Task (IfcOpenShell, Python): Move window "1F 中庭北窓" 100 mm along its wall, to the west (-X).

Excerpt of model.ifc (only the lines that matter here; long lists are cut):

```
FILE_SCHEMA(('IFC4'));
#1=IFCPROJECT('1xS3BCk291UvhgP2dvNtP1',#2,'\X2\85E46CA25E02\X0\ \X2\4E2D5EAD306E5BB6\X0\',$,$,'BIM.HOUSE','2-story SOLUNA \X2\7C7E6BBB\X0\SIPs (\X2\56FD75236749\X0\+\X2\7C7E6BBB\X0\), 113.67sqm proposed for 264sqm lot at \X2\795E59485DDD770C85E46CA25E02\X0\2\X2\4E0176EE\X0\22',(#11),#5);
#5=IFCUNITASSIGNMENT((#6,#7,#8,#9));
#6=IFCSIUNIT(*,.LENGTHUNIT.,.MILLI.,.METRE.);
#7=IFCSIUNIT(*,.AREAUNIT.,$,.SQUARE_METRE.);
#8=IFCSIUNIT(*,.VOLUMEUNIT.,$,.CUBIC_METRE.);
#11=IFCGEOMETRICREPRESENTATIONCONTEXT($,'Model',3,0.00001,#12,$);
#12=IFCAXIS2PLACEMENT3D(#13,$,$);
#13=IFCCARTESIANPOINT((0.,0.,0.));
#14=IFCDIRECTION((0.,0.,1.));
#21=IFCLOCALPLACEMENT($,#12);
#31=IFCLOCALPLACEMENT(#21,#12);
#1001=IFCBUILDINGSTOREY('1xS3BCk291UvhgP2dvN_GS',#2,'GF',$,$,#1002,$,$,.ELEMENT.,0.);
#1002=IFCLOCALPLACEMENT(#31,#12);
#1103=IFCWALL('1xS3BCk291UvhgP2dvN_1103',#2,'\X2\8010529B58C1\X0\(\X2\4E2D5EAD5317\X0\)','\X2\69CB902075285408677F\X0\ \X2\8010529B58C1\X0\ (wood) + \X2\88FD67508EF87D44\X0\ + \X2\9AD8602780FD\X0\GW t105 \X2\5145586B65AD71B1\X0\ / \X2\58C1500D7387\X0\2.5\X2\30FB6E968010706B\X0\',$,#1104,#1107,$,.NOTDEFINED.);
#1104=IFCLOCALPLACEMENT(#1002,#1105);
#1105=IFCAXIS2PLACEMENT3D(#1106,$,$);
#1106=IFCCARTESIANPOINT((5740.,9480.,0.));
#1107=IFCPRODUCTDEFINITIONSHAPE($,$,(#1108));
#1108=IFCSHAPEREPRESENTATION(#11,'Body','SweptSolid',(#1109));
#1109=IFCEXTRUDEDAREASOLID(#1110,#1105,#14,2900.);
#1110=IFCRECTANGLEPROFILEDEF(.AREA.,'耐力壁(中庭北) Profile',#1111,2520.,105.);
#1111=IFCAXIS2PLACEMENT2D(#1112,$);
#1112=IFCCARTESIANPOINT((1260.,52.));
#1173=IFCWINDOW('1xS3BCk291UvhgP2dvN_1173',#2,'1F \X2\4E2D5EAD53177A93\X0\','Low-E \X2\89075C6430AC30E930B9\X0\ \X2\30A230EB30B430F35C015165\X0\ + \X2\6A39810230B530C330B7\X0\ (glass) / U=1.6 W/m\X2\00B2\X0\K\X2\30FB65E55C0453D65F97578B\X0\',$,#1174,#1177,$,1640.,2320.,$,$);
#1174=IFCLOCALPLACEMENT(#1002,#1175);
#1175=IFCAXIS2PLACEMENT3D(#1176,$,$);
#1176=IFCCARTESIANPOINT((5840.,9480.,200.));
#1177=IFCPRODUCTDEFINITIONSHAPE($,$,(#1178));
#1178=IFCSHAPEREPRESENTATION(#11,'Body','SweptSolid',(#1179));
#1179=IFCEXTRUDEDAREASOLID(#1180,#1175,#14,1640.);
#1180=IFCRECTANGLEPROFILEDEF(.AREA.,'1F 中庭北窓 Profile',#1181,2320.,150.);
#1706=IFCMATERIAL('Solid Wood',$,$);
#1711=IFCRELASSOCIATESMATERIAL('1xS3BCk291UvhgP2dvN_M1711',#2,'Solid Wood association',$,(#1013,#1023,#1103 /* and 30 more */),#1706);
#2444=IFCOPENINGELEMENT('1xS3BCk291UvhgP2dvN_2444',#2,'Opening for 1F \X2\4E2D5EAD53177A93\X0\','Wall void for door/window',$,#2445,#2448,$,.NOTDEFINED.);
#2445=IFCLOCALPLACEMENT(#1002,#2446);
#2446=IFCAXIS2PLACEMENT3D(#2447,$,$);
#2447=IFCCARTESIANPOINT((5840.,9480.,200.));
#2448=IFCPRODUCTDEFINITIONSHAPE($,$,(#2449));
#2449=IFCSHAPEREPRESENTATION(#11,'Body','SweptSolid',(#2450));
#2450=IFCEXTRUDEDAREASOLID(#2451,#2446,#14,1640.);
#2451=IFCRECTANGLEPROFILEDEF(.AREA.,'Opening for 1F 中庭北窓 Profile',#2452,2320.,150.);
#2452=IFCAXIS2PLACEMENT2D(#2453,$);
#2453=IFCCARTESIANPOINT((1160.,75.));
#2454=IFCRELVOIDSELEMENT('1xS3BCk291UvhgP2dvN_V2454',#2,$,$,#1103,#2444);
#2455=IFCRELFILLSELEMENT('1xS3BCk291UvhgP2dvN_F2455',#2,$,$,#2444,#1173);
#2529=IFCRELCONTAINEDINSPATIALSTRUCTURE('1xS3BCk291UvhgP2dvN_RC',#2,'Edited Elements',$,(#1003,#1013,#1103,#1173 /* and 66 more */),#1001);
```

```python
import ifcopenshell
import ifcopenshell.api.geometry
import ifcopenshell.util.placement

model = ifcopenshell.open("model.ifc")

window = model.by_id(1173)
opening = window.FillsVoids[0].RelatingOpeningElement
wall = opening.VoidsElements[0].RelatingBuildingElement

wall_matrix = ifcopenshell.util.placement.get_local_placement(wall.ObjectPlacement)
shift = wall_matrix[:3, 0] * -100.0
before = ifcopenshell.util.placement.get_local_placement(window.ObjectPlacement)[:3, 3].copy()

# The window is not placed relative to its opening, so move both.
for product in (opening, window):
    matrix = ifcopenshell.util.placement.get_local_placement(product.ObjectPlacement)
    matrix[:3, 3] += shift
    ifcopenshell.api.geometry.edit_object_placement(model, product=product, matrix=matrix, is_si=False)

after = ifcopenshell.util.placement.get_local_placement(window.ObjectPlacement)[:3, 3]
print("window moved by", (after - before).round(3) + 0.0)

model.write("model-out.ifc")
```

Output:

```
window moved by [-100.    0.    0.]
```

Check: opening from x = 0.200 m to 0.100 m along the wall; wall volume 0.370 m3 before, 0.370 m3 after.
